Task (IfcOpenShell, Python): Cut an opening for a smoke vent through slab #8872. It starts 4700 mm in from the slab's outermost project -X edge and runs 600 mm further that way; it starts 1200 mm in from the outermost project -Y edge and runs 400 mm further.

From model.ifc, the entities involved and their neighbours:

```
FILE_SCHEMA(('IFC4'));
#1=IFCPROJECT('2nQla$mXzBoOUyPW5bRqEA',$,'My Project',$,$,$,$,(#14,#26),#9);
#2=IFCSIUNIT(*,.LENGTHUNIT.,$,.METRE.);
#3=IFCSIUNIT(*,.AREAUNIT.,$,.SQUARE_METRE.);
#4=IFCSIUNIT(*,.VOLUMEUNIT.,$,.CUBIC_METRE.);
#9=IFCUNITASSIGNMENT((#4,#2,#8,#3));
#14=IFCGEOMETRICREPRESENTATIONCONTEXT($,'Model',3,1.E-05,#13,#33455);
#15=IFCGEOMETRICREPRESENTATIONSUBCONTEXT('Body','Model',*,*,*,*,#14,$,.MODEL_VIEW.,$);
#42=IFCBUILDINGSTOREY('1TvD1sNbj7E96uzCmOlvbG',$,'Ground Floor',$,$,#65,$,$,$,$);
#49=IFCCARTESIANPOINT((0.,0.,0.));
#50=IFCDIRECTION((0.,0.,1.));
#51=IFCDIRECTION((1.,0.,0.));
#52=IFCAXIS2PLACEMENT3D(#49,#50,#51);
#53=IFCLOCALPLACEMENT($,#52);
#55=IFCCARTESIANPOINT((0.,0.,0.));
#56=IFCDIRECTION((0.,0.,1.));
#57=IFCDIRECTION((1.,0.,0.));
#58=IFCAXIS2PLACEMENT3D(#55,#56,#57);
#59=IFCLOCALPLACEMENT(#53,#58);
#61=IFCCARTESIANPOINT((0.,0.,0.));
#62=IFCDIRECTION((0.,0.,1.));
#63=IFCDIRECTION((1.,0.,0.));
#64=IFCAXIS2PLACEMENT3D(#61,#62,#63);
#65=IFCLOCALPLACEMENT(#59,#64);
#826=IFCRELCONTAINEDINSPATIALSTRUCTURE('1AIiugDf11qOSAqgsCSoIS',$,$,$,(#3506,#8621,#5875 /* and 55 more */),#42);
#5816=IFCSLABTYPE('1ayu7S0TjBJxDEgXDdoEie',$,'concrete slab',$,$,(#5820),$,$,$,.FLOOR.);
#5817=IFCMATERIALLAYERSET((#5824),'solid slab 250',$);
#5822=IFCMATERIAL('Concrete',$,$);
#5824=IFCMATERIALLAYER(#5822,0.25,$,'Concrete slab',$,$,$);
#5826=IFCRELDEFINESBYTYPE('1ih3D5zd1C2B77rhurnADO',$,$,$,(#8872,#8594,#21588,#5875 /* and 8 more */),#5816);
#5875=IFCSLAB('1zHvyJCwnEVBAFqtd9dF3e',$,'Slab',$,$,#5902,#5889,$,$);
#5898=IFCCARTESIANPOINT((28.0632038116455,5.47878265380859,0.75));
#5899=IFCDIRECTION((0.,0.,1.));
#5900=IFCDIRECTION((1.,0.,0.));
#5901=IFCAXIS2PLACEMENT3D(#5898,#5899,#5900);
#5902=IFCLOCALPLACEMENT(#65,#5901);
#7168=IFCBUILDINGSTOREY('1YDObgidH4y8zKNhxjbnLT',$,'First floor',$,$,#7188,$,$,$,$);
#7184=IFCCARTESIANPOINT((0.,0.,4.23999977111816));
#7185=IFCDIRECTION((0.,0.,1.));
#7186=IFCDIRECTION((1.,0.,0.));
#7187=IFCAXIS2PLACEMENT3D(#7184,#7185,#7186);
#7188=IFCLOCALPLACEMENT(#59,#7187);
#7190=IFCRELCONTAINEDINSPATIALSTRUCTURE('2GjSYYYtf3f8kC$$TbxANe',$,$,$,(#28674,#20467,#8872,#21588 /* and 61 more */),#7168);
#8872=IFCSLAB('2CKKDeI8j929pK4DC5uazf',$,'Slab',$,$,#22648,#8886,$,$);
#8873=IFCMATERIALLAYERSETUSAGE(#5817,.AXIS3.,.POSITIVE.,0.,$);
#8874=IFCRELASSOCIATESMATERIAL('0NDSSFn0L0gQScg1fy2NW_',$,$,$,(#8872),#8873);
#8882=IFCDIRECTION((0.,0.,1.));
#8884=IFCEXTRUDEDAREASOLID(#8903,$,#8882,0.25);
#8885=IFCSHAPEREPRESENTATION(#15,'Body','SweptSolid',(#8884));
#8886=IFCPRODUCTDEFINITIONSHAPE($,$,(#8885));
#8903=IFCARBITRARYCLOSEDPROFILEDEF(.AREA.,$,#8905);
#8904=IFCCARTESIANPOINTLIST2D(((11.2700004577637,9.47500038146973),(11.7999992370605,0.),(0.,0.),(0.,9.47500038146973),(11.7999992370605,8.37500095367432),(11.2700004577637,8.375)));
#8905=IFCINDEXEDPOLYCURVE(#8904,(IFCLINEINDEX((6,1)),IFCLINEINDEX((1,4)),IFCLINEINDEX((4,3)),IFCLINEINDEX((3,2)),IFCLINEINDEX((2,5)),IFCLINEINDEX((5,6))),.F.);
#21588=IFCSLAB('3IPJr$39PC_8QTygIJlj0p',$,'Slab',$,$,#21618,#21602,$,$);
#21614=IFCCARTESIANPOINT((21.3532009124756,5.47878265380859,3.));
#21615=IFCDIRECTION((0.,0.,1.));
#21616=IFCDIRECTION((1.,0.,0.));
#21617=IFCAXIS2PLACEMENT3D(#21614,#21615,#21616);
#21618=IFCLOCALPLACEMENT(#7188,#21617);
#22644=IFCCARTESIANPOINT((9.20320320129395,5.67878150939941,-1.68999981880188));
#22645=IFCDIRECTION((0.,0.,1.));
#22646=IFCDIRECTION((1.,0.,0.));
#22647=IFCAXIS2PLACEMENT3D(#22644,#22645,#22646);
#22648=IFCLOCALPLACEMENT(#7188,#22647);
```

```python
import numpy as np
import ifcopenshell
import ifcopenshell.api.feature
import ifcopenshell.api.geometry
import ifcopenshell.api.root
import ifcopenshell.geom
import ifcopenshell.util.placement
import ifcopenshell.util.representation
import ifcopenshell.util.shape
import ifcopenshell.util.unit

model = ifcopenshell.open("model.ifc")
unit_scale = ifcopenshell.util.unit.calculate_unit_scale(model)
settings = ifcopenshell.geom.settings()


def volume(element):
    """Net volume in cubic metres, openings subtracted."""
    shape = ifcopenshell.geom.create_shape(settings, element)
    return ifcopenshell.util.shape.get_volume(shape.geometry)


slab = model.by_id(8872)
before = volume(slab)

# Extent in the slab's own axes, in metres. The edges named are its -X and -Y sides.
slab_shape = ifcopenshell.geom.create_shape(settings, slab)
vertices = ifcopenshell.util.shape.get_vertices(slab_shape.geometry)
x_min, y_min, bottom = vertices.min(axis=0)
top = vertices[:, 2].max()

opening = ifcopenshell.api.root.create_entity(model, ifc_class="IfcOpeningElement", name="Smoke vent opening", predefined_type="OPENING")
context = ifcopenshell.util.representation.get_context(model, "Model", "Body", "MODEL_VIEW")
width, depth = 0.6, 0.4
outline = [(0.0, 0.0), (width, 0.0), (width, depth), (0.0, depth), (0.0, 0.0)]
# Overshoot both faces by 50 mm so the cut is clean.
shape = ifcopenshell.api.geometry.add_slab_representation(
    model, context=context, depth=top - bottom + 0.1, polyline=outline
)
ifcopenshell.api.geometry.assign_representation(model, product=opening, representation=shape)

matrix = ifcopenshell.util.placement.get_local_placement(slab.ObjectPlacement)
matrix[:, 3] = matrix @ np.append(np.array([x_min + 4.7, y_min + 1.2, bottom - 0.05]) / unit_scale, 1.0)
ifcopenshell.api.geometry.edit_object_placement(model, product=opening, matrix=matrix, is_si=False)
ifcopenshell.api.feature.add_feature(model, feature=opening, element=slab)

after = volume(slab)

print(f"slab volume {before:.3f} -> {after:.3f} m3")

model.write("model_edited.ifc")
```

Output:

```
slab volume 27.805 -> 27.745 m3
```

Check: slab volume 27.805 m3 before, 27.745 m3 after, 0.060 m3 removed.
